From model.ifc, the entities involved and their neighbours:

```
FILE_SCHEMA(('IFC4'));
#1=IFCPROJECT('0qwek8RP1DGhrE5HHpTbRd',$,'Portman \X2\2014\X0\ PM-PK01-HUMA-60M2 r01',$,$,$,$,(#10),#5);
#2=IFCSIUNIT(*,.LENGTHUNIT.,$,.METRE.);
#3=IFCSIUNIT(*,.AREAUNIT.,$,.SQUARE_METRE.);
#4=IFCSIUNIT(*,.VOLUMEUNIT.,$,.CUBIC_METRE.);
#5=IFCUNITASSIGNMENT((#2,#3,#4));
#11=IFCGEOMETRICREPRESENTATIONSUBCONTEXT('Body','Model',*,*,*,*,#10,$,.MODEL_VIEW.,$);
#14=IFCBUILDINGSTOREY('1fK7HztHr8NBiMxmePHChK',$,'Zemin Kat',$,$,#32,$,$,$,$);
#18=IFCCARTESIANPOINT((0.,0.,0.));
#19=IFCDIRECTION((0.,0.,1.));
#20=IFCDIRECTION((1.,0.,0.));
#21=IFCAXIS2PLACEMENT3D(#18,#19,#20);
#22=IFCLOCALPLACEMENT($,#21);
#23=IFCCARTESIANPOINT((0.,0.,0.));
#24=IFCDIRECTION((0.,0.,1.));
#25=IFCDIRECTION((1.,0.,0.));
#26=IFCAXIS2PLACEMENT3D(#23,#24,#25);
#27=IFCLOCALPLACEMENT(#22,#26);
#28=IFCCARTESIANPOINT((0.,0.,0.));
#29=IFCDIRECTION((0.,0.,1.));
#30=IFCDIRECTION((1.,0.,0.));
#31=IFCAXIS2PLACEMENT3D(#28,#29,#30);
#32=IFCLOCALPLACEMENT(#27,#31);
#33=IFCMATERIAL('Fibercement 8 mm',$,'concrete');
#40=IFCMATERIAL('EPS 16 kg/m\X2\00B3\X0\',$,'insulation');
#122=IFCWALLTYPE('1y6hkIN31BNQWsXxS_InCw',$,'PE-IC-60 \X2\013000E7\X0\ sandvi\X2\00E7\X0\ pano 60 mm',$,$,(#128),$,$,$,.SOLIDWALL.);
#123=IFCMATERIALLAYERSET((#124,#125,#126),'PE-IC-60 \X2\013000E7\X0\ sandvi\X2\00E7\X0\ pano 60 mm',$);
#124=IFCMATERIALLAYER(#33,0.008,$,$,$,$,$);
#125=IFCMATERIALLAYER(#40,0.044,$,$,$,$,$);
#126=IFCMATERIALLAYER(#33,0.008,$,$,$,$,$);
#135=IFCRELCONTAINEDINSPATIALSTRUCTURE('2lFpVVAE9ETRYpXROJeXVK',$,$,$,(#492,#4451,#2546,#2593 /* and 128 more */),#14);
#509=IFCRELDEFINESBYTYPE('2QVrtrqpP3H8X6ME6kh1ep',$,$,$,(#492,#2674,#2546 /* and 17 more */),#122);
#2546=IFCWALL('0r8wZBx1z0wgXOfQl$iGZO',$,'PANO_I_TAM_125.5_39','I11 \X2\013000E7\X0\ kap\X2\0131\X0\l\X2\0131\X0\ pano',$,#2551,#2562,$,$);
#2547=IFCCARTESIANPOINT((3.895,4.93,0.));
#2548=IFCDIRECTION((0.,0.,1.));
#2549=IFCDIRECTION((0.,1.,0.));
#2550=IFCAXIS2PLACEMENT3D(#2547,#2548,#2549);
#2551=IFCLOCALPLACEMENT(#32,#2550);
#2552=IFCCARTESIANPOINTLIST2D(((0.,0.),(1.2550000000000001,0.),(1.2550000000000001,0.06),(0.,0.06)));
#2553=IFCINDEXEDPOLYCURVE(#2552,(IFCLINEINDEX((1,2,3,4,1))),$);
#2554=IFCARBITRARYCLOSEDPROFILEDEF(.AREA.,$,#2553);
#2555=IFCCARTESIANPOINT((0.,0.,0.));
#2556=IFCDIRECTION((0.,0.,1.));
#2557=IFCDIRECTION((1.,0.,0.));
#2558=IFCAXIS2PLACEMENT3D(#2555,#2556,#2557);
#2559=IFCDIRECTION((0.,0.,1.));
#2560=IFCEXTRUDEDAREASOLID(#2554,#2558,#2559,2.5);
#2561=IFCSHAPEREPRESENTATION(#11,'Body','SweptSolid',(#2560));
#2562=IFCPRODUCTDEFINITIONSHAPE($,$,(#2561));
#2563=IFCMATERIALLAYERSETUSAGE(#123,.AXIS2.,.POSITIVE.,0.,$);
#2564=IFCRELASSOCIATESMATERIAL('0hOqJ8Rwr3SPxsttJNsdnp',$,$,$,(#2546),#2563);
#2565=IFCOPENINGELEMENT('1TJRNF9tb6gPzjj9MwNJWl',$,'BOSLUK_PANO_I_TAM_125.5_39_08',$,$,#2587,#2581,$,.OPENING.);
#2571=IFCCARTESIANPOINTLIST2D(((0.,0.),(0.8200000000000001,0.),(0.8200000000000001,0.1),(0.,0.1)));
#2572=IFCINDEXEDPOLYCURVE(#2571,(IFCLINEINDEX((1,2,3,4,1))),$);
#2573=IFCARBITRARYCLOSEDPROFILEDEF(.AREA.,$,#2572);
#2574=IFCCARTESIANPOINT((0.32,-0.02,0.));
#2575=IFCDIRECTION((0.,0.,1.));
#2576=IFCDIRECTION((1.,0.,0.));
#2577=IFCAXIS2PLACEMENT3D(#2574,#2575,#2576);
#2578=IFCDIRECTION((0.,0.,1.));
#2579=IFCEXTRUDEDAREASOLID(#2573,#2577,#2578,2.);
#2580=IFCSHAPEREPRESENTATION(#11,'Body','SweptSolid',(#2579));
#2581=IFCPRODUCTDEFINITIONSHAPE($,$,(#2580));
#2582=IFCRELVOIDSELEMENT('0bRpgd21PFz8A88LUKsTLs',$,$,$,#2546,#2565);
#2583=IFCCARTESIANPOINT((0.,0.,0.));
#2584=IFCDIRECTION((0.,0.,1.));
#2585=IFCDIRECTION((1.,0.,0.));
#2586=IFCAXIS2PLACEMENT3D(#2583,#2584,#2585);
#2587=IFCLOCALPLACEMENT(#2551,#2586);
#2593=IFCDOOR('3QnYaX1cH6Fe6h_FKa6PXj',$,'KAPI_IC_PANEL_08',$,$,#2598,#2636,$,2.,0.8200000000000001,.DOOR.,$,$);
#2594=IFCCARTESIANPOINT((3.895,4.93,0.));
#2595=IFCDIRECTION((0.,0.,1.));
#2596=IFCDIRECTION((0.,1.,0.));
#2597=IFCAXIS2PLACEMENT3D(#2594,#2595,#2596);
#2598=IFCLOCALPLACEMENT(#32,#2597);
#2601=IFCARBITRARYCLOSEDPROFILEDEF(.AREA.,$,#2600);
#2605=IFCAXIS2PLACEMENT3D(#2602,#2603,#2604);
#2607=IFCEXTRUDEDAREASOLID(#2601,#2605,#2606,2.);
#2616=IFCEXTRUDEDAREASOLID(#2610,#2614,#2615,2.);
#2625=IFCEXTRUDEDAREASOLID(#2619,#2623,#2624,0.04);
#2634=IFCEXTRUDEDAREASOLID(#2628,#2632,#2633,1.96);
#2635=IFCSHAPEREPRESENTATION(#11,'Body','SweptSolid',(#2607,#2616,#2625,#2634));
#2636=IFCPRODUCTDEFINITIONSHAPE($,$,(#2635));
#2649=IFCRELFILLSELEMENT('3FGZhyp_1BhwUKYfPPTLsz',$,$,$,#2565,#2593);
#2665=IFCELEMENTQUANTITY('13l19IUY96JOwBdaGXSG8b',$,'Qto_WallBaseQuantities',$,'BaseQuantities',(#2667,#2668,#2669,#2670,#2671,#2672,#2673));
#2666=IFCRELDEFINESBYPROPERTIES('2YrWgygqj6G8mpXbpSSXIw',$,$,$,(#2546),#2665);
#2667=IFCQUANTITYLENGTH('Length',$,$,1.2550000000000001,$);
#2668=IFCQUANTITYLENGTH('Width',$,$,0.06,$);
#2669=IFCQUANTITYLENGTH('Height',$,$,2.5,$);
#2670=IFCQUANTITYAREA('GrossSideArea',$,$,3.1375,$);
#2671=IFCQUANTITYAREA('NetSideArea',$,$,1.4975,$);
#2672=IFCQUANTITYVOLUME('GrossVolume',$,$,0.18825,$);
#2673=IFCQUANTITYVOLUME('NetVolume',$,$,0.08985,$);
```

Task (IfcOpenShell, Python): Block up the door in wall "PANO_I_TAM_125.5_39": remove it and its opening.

```python
import ifcopenshell
import ifcopenshell.api.feature
import ifcopenshell.api.pset
import ifcopenshell.api.root
import ifcopenshell.geom
import ifcopenshell.util.element
import ifcopenshell.util.shape
import ifcopenshell.util.unit

model = ifcopenshell.open("model.ifc")
area_scale = ifcopenshell.util.unit.calculate_unit_scale(model, "AREAUNIT")
volume_scale = ifcopenshell.util.unit.calculate_unit_scale(model, "VOLUMEUNIT")
settings = ifcopenshell.geom.settings()


def volume(element):
    """Net volume in cubic metres, openings subtracted."""
    shape = ifcopenshell.geom.create_shape(settings, element)
    return ifcopenshell.util.shape.get_volume(shape.geometry)


door = model.by_guid("3QnYaX1cH6Fe6h_FKa6PXj")
opening = door.FillsVoids[0].RelatingOpeningElement
wall = opening.VoidsElements[0].RelatingBuildingElement
before = volume(wall)

ifcopenshell.api.root.remove_product(model, product=door)
ifcopenshell.api.feature.remove_feature(model, feature=opening)

after = volume(wall)
thickness = 0.06  # wall thickness in metres

# Update the wall's stored quantities.
qto = model.by_id(ifcopenshell.util.element.get_pset(wall, "Qto_WallBaseQuantities", should_inherit=False)["id"])
ifcopenshell.api.pset.edit_qto(model, qto=qto, properties={
    "NetSideArea": after / thickness / area_scale,
    "NetVolume": after / volume_scale,
})

print(f"wall volume {before:.3f} -> {after:.3f} m3")

model.write("model_v2.ifc")
```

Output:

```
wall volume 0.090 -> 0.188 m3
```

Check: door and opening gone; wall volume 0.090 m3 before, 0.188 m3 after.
